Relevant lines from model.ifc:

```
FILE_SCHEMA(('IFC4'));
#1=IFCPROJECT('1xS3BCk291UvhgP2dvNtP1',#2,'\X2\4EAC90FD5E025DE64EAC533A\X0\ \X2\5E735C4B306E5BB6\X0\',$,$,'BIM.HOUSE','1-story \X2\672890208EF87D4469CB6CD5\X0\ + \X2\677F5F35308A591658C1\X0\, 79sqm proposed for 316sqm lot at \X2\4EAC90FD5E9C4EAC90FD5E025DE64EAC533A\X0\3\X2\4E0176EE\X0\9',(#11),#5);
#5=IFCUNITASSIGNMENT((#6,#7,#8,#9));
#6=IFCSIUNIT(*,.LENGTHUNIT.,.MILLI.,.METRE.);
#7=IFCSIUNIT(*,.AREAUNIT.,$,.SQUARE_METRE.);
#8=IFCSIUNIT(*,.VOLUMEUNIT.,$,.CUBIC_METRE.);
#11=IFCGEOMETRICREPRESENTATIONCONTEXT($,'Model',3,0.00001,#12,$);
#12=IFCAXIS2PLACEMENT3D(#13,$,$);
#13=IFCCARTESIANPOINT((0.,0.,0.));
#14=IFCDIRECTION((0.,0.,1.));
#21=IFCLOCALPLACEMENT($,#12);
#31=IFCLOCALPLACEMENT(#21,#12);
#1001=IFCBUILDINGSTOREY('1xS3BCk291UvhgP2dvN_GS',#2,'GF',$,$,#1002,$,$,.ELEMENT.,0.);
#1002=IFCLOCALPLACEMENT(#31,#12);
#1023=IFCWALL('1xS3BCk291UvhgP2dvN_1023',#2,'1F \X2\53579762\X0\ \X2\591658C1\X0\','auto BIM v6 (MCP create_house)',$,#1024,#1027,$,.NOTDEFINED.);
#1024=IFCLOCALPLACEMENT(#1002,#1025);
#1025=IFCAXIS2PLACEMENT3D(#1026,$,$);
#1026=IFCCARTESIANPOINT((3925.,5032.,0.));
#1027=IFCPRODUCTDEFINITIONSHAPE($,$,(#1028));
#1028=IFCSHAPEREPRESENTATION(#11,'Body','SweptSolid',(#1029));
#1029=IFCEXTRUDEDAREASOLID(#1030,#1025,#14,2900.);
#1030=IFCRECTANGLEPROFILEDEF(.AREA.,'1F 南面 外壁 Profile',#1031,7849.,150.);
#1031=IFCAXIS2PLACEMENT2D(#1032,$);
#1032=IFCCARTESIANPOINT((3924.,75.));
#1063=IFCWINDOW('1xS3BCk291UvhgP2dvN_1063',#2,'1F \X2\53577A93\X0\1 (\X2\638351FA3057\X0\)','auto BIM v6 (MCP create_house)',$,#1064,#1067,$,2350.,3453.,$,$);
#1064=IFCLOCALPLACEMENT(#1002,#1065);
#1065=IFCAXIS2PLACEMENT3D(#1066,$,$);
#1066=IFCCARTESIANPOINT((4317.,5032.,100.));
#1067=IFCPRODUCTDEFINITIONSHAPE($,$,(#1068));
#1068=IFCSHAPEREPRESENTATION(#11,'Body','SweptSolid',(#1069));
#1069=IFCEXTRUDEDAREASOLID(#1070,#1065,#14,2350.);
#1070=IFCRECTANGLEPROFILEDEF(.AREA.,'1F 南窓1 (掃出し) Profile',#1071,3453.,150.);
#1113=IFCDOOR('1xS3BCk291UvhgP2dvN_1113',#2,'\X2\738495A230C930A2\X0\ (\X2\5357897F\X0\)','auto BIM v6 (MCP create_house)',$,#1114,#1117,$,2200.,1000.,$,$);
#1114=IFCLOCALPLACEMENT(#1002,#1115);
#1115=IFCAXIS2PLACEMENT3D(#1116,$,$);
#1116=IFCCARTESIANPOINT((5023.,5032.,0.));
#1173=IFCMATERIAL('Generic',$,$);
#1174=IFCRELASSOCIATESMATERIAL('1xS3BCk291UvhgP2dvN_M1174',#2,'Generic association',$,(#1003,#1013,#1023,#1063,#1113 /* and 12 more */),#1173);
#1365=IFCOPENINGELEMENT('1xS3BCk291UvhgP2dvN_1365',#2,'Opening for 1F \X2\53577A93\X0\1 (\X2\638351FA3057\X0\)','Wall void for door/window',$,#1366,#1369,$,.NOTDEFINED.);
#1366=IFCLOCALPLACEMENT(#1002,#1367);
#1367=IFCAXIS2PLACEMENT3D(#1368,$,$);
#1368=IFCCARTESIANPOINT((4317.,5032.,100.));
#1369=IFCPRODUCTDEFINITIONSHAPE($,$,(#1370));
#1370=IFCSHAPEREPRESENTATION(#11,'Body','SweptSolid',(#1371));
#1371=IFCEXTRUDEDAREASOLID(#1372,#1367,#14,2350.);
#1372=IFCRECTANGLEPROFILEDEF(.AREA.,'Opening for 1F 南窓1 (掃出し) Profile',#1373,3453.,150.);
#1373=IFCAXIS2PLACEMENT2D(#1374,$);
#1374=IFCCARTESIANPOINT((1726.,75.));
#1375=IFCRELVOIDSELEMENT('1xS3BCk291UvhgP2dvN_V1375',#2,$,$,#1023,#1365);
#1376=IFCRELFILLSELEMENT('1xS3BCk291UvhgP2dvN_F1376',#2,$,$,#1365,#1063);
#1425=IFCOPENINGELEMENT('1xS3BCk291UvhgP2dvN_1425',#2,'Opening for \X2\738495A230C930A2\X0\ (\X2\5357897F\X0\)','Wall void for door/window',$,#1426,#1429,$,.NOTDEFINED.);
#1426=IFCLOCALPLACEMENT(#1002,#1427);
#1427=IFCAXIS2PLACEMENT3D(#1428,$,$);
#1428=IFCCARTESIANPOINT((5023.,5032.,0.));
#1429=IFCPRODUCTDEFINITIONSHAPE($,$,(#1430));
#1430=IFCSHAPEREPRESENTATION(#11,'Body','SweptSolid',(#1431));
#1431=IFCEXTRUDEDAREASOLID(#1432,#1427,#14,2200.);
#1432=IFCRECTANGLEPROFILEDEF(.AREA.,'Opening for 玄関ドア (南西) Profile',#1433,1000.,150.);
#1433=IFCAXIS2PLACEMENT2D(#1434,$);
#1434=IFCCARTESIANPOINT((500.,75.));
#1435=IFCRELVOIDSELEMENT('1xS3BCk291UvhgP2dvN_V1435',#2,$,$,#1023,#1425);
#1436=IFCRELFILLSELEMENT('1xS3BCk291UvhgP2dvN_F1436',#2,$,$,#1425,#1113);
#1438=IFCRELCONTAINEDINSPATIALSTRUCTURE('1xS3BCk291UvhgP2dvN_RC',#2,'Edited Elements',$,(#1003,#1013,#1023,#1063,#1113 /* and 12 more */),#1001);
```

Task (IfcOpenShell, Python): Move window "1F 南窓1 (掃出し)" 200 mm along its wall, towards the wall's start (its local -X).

```python
import ifcopenshell
import ifcopenshell.api.geometry
import ifcopenshell.util.placement

model = ifcopenshell.open("model.ifc")

window = model.by_guid("1xS3BCk291UvhgP2dvN_1063")
opening = window.FillsVoids[0].RelatingOpeningElement
wall = opening.VoidsElements[0].RelatingBuildingElement

wall_matrix = ifcopenshell.util.placement.get_local_placement(wall.ObjectPlacement)
shift = wall_matrix[:3, 0] * -200.0
before = ifcopenshell.util.placement.get_local_placement(window.ObjectPlacement)[:3, 3].copy()

# The window is not placed relative to its opening, so move both.
for product in (opening, window):
    matrix = ifcopenshell.util.placement.get_local_placement(product.ObjectPlacement)
    matrix[:3, 3] += shift
    ifcopenshell.api.geometry.edit_object_placement(model, product=product, matrix=matrix, is_si=False)

after = ifcopenshell.util.placement.get_local_placement(window.ObjectPlacement)[:3, 3]
print("window moved by", (after - before).round(3) + 0.0)

model.write("model_v2.ifc")
```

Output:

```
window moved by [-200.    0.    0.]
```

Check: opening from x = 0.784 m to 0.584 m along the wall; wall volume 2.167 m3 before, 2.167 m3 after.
